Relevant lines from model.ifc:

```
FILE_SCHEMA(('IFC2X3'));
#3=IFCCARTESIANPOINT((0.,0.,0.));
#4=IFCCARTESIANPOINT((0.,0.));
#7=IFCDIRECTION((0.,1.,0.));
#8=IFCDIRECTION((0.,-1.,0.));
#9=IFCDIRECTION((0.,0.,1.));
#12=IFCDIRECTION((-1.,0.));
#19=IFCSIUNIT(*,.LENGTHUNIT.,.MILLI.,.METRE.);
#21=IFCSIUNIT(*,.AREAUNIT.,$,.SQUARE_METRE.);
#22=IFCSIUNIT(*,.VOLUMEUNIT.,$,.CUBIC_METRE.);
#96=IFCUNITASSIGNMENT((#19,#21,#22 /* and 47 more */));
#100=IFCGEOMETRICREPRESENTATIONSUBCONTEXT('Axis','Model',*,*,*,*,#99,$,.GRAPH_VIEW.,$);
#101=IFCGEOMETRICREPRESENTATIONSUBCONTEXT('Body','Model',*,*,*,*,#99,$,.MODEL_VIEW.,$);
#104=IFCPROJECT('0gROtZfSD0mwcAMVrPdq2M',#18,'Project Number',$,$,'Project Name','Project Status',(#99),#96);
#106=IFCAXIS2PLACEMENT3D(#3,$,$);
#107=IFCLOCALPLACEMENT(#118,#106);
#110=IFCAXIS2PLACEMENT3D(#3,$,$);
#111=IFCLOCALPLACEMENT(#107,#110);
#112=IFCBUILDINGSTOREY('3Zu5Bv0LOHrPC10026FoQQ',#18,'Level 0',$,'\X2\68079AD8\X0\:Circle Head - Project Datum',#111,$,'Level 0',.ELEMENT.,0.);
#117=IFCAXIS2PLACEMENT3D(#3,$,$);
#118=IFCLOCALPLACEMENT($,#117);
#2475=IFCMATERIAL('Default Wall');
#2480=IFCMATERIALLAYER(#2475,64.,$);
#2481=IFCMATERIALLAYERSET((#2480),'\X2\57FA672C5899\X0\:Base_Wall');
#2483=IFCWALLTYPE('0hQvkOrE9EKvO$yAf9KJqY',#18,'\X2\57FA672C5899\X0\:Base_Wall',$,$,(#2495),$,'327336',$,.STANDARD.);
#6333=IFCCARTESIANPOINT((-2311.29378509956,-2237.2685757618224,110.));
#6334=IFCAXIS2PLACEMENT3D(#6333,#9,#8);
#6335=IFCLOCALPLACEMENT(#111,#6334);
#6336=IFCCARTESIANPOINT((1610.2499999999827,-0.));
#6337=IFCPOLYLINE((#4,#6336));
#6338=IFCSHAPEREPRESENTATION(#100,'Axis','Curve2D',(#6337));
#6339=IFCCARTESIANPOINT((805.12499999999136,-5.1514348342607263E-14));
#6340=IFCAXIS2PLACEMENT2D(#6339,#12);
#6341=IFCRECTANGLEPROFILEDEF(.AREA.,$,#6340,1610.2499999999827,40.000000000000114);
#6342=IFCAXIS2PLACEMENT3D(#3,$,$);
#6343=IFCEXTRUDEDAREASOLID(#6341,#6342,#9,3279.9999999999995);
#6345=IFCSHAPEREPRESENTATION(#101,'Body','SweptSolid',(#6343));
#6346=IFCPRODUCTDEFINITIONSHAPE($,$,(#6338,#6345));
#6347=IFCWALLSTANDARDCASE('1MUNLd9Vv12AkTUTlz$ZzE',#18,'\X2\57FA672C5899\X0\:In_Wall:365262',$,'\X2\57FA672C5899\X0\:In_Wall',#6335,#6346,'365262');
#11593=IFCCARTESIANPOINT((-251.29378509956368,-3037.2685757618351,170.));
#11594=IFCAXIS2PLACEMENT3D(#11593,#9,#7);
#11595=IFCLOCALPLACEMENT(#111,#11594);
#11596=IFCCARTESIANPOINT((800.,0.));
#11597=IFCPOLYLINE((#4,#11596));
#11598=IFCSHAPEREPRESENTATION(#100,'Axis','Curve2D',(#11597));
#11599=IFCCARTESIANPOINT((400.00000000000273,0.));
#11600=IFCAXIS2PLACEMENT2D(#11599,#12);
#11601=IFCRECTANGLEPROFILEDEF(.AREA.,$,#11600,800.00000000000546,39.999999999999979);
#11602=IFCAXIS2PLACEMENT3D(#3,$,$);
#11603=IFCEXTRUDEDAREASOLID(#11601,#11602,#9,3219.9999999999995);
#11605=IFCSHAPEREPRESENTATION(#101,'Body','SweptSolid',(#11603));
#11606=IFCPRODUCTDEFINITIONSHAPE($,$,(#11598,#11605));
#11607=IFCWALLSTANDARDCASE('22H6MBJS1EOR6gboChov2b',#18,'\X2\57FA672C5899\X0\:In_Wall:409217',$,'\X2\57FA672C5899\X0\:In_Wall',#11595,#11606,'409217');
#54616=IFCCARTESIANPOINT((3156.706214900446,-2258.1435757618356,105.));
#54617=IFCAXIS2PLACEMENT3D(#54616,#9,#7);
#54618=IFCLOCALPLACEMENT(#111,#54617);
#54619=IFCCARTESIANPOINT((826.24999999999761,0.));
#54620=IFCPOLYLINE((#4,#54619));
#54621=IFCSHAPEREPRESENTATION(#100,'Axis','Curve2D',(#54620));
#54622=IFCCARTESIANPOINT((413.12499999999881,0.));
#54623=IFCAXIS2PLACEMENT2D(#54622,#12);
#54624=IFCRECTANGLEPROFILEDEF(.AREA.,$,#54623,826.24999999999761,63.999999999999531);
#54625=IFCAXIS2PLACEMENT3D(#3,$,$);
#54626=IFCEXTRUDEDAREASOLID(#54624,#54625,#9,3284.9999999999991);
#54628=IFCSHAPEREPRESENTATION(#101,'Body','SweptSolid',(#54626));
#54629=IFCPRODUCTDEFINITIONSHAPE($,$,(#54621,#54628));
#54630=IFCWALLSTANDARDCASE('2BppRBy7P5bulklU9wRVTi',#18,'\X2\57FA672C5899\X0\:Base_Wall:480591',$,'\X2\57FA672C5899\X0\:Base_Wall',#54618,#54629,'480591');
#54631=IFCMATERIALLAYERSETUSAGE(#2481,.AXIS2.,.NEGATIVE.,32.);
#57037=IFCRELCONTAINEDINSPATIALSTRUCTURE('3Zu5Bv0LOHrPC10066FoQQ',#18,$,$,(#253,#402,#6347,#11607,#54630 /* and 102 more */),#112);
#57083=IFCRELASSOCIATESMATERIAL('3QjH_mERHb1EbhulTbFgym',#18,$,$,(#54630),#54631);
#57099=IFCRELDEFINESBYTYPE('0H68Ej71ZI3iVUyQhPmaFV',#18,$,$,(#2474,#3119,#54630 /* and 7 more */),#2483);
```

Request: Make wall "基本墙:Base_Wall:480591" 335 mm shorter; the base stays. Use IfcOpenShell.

```python
import ifcopenshell
import ifcopenshell.geom
import ifcopenshell.util.representation
import ifcopenshell.util.shape
import ifcopenshell.util.unit

model = ifcopenshell.open("model.ifc")
unit_scale = ifcopenshell.util.unit.calculate_unit_scale(model)
settings = ifcopenshell.geom.settings()


def volume(element):
    """Net volume in cubic metres, openings subtracted."""
    shape = ifcopenshell.geom.create_shape(settings, element)
    return ifcopenshell.util.shape.get_volume(shape.geometry)


wall = model.by_guid("2BppRBy7P5bulklU9wRVTi")
before = volume(wall)

body = ifcopenshell.util.representation.get_representation(wall, "Model", "Body")
solid = body.Items[0]
old_height = solid.Depth
solid.Depth -= 0.335 / unit_scale
after = volume(wall)

print(f"height {old_height:g} -> {solid.Depth:g}, volume {before:.3f} -> {after:.3f} m3")

model.write("model_v2.ifc")
```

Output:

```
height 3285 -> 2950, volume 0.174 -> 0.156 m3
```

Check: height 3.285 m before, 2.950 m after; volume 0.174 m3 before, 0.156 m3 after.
